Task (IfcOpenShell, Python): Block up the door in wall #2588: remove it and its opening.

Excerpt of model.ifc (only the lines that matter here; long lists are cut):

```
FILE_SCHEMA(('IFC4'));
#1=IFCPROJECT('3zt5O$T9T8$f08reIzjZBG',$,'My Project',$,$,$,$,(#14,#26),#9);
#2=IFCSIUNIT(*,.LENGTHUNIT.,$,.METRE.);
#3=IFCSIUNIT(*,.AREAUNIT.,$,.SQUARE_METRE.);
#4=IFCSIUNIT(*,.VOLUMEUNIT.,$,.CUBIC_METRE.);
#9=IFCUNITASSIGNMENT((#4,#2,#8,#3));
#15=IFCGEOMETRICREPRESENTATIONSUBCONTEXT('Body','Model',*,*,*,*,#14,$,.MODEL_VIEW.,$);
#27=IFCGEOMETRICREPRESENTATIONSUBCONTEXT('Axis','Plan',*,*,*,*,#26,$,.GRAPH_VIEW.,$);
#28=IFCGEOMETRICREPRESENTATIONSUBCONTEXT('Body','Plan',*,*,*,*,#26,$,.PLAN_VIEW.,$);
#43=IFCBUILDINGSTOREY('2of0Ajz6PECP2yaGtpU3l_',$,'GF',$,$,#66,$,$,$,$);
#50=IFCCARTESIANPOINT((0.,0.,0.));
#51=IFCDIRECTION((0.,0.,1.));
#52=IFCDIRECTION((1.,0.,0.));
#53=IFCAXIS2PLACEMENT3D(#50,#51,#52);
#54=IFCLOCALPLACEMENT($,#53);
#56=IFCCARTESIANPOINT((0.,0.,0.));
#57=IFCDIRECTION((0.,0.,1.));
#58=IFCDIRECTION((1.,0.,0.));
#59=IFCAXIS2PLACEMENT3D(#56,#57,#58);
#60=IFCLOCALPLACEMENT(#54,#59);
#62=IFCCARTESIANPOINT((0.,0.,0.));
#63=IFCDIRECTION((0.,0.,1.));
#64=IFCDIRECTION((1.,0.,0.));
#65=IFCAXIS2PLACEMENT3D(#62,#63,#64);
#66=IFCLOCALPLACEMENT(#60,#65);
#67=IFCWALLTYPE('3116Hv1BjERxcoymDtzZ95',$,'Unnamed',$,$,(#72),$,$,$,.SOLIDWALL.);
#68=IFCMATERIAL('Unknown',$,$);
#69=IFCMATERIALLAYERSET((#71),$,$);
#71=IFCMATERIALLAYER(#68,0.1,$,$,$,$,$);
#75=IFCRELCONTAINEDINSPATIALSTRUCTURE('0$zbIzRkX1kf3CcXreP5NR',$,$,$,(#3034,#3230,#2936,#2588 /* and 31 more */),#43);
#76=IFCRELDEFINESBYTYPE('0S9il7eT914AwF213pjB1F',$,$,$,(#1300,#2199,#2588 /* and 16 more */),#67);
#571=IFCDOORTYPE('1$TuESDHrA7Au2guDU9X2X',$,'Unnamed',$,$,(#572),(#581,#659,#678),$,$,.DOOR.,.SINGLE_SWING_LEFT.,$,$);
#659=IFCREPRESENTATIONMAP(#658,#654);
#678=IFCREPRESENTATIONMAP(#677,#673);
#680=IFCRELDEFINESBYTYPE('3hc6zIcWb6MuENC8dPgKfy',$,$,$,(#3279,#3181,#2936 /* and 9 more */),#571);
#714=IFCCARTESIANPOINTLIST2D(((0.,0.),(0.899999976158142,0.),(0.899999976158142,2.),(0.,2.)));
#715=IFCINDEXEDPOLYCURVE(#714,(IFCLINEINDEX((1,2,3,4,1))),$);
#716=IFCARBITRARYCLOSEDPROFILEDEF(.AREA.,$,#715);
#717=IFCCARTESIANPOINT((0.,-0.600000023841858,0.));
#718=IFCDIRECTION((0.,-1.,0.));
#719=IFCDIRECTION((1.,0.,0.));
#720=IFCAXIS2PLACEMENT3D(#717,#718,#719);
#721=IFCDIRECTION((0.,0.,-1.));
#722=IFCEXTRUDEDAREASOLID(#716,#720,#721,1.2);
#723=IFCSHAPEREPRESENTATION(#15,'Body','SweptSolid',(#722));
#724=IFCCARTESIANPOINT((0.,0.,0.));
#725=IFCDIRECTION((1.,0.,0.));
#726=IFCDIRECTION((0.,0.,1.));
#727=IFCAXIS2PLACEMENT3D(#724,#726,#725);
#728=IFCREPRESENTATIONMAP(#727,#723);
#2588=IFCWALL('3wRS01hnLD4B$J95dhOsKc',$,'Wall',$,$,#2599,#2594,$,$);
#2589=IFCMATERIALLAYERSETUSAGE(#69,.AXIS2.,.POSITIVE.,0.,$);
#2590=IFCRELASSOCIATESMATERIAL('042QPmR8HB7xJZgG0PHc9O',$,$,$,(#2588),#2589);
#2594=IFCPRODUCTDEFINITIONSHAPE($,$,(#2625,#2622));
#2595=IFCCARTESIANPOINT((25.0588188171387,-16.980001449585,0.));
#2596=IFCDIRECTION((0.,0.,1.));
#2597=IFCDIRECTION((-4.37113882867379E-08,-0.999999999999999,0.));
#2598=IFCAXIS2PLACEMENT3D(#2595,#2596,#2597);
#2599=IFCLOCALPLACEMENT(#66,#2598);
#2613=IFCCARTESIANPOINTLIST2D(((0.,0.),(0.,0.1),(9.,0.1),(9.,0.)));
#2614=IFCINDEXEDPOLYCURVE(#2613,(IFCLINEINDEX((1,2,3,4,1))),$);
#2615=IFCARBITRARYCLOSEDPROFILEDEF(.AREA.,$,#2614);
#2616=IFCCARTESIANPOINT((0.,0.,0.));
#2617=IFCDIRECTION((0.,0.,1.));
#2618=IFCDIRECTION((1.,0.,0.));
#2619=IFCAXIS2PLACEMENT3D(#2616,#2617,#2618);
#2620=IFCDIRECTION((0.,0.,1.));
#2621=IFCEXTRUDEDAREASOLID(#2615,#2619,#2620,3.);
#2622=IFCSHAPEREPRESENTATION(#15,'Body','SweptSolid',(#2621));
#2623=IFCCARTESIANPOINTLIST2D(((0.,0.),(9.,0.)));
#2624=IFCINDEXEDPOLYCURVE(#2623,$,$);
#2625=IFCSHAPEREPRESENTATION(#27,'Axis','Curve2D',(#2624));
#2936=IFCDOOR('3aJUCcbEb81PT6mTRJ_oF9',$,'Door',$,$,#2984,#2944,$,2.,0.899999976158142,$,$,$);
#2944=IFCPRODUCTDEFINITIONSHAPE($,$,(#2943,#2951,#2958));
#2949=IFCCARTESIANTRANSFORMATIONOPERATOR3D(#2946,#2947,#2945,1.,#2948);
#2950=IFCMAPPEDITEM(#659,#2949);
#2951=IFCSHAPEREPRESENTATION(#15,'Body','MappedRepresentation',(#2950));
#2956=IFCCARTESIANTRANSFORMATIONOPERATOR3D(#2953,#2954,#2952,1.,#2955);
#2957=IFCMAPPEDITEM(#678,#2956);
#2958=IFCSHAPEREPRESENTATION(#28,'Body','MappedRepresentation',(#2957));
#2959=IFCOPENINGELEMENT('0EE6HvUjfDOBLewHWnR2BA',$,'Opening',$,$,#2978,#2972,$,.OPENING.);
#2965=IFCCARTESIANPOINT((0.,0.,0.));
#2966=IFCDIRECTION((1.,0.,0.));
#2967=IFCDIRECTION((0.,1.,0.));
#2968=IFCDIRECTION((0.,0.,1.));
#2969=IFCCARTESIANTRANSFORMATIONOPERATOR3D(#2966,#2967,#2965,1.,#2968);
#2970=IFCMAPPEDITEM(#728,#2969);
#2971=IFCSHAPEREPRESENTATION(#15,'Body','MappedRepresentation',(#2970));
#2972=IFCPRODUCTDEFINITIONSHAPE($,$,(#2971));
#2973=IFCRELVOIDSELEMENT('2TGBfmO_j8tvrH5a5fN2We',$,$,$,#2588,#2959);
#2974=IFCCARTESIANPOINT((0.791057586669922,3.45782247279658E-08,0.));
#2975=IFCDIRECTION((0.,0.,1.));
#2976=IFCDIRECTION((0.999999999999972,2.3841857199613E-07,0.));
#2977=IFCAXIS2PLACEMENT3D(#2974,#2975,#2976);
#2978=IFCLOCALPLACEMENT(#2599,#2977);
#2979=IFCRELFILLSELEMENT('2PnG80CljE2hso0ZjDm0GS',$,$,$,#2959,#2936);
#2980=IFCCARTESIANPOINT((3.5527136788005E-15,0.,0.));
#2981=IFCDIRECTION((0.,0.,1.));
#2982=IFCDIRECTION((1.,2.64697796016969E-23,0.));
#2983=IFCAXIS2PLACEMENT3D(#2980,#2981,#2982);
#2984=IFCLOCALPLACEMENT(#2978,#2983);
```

```python
import ifcopenshell
import ifcopenshell.api.feature
import ifcopenshell.api.root
import ifcopenshell.geom
import ifcopenshell.util.shape

model = ifcopenshell.open("model.ifc")
settings = ifcopenshell.geom.settings()


def volume(element):
    """Net volume in cubic metres, openings subtracted."""
    shape = ifcopenshell.geom.create_shape(settings, element)
    return ifcopenshell.util.shape.get_volume(shape.geometry)


door = model.by_id(2936)
opening = door.FillsVoids[0].RelatingOpeningElement
wall = opening.VoidsElements[0].RelatingBuildingElement
before = volume(wall)

ifcopenshell.api.root.remove_product(model, product=door)
ifcopenshell.api.feature.remove_feature(model, feature=opening)

after = volume(wall)

print(f"wall volume {before:.3f} -> {after:.3f} m3")

model.write("model_rev.ifc")
```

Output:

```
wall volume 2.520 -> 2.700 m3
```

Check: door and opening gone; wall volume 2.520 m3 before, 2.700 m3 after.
